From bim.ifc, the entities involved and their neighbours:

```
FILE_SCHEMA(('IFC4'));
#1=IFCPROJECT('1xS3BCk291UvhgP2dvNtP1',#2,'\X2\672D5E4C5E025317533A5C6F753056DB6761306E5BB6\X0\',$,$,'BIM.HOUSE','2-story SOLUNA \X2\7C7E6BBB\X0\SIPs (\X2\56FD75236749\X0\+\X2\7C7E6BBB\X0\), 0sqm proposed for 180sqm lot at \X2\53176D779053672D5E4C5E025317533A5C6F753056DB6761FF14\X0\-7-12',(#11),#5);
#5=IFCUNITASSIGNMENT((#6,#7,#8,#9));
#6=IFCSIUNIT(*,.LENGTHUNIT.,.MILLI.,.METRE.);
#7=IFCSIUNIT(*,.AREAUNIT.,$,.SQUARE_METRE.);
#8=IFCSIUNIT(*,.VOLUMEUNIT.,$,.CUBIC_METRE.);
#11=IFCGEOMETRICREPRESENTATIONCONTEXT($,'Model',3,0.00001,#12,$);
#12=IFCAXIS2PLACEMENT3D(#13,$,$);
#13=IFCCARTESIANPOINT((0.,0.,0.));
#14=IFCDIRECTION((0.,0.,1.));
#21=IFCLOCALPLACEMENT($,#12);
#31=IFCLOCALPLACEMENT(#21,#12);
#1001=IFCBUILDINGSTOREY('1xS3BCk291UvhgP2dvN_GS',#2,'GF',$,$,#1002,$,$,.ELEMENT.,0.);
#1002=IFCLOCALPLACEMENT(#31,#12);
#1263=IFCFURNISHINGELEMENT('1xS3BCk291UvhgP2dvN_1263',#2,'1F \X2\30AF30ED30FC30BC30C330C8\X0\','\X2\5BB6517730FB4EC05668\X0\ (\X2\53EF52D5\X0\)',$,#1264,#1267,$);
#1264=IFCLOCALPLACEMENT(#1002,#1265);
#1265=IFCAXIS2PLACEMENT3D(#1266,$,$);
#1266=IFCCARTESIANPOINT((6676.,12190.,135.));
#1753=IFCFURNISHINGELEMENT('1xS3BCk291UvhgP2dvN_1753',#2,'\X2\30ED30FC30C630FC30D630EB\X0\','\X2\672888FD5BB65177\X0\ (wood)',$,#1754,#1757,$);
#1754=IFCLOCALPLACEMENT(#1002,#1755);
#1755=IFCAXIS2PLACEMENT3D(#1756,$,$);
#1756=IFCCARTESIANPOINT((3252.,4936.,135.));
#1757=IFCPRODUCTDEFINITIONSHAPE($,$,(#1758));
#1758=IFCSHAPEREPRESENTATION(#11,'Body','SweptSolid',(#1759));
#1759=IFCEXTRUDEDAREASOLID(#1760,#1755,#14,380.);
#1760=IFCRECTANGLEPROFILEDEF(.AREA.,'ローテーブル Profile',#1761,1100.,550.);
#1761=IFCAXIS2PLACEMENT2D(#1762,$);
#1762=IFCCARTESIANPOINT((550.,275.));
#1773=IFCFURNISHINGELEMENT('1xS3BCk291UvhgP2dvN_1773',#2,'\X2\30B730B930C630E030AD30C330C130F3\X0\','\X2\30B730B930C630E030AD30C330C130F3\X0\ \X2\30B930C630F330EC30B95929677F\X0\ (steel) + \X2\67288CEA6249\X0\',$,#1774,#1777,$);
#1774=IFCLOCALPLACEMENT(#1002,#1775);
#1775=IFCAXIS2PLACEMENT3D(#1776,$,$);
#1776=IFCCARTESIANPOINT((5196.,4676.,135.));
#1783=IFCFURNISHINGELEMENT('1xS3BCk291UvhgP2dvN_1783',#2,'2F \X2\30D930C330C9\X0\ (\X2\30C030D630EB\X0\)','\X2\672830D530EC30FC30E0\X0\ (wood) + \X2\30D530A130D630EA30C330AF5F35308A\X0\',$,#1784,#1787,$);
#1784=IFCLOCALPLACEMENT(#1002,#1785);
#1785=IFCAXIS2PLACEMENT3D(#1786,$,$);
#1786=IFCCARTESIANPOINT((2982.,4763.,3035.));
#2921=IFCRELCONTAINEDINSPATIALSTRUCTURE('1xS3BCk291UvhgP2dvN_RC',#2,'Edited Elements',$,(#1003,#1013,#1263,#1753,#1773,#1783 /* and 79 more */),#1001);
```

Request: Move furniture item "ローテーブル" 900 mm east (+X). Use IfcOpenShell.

```python
import ifcopenshell
import ifcopenshell.api.geometry
import ifcopenshell.util.placement
import ifcopenshell.util.unit

model = ifcopenshell.open("bim.ifc")
unit_scale = ifcopenshell.util.unit.calculate_unit_scale(model)

item = model.by_guid("1xS3BCk291UvhgP2dvN_1753")
matrix = ifcopenshell.util.placement.get_local_placement(item.ObjectPlacement)
matrix[0, 3] += 0.9 / unit_scale
ifcopenshell.api.geometry.edit_object_placement(model, product=item, matrix=matrix, is_si=False)

print(ifcopenshell.util.placement.get_local_placement(item.ObjectPlacement).round(3) + 0.0)

model.write("bim_edited.ifc")
```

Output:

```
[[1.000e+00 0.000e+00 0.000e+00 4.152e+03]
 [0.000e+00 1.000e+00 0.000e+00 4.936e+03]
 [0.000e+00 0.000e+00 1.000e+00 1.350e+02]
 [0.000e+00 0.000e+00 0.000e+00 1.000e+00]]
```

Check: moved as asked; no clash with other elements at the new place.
